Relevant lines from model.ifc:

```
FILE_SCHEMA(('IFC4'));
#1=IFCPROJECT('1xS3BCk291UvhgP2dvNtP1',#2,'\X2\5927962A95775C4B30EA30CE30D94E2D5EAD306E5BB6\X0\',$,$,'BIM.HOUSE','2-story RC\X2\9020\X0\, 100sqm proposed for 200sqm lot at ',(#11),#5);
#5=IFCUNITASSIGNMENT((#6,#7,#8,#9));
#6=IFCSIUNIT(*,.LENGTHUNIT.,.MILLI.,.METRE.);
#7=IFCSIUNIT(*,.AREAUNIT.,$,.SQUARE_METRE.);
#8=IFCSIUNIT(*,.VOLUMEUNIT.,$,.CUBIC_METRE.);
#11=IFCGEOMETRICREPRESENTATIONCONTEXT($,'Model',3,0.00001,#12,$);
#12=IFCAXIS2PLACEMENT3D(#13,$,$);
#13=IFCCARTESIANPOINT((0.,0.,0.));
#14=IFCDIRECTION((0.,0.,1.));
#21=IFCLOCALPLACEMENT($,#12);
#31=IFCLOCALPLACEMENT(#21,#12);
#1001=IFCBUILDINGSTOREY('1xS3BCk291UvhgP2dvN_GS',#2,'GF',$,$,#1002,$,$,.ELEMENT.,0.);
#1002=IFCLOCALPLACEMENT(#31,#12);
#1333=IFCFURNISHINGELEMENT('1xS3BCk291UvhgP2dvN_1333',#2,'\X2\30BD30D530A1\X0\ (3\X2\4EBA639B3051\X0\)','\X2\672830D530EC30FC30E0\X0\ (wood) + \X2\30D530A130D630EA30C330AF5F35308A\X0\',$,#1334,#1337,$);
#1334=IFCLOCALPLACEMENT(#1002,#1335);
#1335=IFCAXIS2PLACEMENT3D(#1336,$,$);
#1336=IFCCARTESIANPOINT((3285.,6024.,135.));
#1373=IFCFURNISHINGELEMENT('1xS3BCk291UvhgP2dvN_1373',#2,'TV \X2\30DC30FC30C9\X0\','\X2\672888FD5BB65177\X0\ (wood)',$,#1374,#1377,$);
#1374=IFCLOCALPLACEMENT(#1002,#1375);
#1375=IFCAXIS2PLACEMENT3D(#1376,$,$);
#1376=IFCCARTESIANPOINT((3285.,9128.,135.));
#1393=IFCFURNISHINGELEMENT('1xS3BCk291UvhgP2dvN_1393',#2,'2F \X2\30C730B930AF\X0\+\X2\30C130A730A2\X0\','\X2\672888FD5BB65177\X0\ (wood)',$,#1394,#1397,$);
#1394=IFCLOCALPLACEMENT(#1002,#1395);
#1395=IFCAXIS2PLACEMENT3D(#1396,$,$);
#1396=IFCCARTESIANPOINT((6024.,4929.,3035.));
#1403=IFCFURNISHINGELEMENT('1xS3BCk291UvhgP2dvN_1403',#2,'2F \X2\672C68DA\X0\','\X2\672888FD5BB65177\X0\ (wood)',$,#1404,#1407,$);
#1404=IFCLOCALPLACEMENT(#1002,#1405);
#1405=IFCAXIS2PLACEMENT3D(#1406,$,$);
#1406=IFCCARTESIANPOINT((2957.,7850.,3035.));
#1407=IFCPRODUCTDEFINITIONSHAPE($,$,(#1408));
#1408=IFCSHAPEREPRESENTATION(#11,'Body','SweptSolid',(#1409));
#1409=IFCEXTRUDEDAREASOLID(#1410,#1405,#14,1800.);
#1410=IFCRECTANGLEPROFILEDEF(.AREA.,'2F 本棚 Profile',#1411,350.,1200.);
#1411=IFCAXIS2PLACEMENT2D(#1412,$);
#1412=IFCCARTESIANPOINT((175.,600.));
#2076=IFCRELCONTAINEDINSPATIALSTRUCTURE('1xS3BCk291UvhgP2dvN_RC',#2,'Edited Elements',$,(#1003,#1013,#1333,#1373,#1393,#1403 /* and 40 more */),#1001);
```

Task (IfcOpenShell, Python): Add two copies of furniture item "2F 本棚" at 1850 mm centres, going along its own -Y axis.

```python
import ifcopenshell
import ifcopenshell.api.geometry
import ifcopenshell.api.root
import ifcopenshell.util.element
import ifcopenshell.util.placement
import ifcopenshell.util.unit

model = ifcopenshell.open("model.ifc")
unit_scale = ifcopenshell.util.unit.calculate_unit_scale(model)


def reuse_history(source, copy):
    """copy_class also copies each property set's owner history, people and application; keep the originals."""
    for rel in copy.IsDefinedBy:
        if rel.is_a("IfcRelDefinesByProperties") and (history := rel.RelatingPropertyDefinition.OwnerHistory):
            rel.RelatingPropertyDefinition.OwnerHistory = source.OwnerHistory
            ifcopenshell.util.element.remove_deep2(model, history)


source = model.by_id(1403)
base = ifcopenshell.util.placement.get_local_placement(source.ObjectPlacement)
step = -base[:3, 1] * 1.85 / unit_scale

for i in range(1, 3):
    copy = ifcopenshell.api.root.copy_class(model, product=source)
    copy.Representation = ifcopenshell.util.element.copy_deep(
        model, source.Representation, exclude=["IfcGeometricRepresentationContext", "IfcRepresentationMap"]
    )
    reuse_history(source, copy)
    matrix = base.copy()
    matrix[:3, 3] += i * step
    print("added at", matrix[:3, 3].round(3) + 0.0)
    ifcopenshell.api.geometry.edit_object_placement(model, product=copy, matrix=matrix, is_si=False)

model.write("model_v2.ifc")
```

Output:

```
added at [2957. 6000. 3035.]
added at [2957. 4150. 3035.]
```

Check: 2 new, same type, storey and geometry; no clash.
